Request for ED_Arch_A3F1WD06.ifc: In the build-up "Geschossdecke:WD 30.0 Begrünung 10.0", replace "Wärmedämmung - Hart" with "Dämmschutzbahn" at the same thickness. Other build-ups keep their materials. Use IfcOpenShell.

First a look at what the model holds.

```python
import ifcopenshell
import ifcopenshell.util.element

model = ifcopenshell.open("ED_Arch_A3F1WD06.ifc")
print(model.schema)
for layer_set in model.by_type("IfcMaterialLayerSet"):
    if layer_set.LayerSetName == "Geschossdecke:WD 30.0 Begrünung 10.0":
        for layer in layer_set.MaterialLayers:
            print(layer.id(), layer.Material and layer.Material.Name, layer.LayerThickness, sep=" | ")
        print(len(ifcopenshell.util.element.get_elements_by_material(model, layer_set)), "elements and types use it")
print(sorted(m.Name for m in model.by_type("IfcMaterial") if m.Name)[:60])
```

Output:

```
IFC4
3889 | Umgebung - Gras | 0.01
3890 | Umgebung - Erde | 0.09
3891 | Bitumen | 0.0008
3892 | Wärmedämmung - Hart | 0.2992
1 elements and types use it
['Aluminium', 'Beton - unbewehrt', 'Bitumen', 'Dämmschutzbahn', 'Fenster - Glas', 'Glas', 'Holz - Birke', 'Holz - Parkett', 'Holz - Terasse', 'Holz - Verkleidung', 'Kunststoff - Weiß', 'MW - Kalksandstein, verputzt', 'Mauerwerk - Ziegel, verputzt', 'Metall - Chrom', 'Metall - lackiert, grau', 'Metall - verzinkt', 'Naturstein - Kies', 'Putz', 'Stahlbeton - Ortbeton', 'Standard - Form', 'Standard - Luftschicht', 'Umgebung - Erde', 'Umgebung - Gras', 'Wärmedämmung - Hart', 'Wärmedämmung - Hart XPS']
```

```python
import ifcopenshell
import ifcopenshell.api.material

model = ifcopenshell.open("ED_Arch_A3F1WD06.ifc")

layer_set = next(s for s in model.by_type("IfcMaterialLayerSet") if s.LayerSetName == "Geschossdecke:WD 30.0 Begrünung 10.0")
layer = next(l for l in layer_set.MaterialLayers if l.Material and l.Material.Name == "Wärmedämmung - Hart")
material = next(m for m in model.by_type("IfcMaterial") if m.Name == "Dämmschutzbahn")

# Point this one layer at the other material; renaming the old one would change it everywhere.
ifcopenshell.api.material.edit_layer(model, layer=layer, attributes={}, material=material)

print([l.Material.Name if l.Material else None for l in layer_set.MaterialLayers])

model.write("ED_Arch_A3F1WD06_updated.ifc")
```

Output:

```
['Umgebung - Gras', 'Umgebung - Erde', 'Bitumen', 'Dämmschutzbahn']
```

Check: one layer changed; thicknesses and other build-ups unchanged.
